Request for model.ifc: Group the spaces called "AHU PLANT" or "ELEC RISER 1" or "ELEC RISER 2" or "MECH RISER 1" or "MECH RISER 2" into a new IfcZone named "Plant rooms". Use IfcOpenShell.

First a look at what the model holds.

```python
import ifcopenshell

model = ifcopenshell.open("model.ifc")
print(model.schema)
seen = {}
for space in model.by_type("IfcSpace"):
    seen[space.LongName] = seen.get(space.LongName, 0) + 1
for name, count in sorted(seen.items(), key=str):
    print(count, "x", name)
print("zones:", [z.Name for z in model.by_type("IfcZone")][:20])
```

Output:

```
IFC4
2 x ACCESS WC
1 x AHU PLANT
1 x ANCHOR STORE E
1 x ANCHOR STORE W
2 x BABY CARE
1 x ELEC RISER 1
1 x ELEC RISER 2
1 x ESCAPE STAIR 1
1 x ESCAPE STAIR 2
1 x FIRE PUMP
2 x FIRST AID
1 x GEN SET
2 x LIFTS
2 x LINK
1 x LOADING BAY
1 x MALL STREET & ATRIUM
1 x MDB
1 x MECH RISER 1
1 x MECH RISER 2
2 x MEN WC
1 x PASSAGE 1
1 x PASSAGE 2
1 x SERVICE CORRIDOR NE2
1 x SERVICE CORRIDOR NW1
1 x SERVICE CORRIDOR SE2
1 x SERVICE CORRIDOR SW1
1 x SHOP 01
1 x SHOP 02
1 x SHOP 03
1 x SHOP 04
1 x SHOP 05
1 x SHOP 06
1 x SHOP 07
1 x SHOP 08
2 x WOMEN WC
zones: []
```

```python
import ifcopenshell
import ifcopenshell.api.group
import ifcopenshell.api.root

model = ifcopenshell.open("model.ifc")

names = {"AHU PLANT", "ELEC RISER 1", "ELEC RISER 2", "MECH RISER 1", "MECH RISER 2"}
spaces = [s for s in model.by_type("IfcSpace") if s.LongName in names]

zone = ifcopenshell.api.root.create_entity(model, ifc_class="IfcZone", name="Plant rooms")
ifcopenshell.api.group.assign_group(model, products=spaces, group=zone)
print(len(spaces), "spaces in", zone.Name)

model.write("model_rev.ifc")
```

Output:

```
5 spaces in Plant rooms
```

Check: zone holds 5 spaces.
